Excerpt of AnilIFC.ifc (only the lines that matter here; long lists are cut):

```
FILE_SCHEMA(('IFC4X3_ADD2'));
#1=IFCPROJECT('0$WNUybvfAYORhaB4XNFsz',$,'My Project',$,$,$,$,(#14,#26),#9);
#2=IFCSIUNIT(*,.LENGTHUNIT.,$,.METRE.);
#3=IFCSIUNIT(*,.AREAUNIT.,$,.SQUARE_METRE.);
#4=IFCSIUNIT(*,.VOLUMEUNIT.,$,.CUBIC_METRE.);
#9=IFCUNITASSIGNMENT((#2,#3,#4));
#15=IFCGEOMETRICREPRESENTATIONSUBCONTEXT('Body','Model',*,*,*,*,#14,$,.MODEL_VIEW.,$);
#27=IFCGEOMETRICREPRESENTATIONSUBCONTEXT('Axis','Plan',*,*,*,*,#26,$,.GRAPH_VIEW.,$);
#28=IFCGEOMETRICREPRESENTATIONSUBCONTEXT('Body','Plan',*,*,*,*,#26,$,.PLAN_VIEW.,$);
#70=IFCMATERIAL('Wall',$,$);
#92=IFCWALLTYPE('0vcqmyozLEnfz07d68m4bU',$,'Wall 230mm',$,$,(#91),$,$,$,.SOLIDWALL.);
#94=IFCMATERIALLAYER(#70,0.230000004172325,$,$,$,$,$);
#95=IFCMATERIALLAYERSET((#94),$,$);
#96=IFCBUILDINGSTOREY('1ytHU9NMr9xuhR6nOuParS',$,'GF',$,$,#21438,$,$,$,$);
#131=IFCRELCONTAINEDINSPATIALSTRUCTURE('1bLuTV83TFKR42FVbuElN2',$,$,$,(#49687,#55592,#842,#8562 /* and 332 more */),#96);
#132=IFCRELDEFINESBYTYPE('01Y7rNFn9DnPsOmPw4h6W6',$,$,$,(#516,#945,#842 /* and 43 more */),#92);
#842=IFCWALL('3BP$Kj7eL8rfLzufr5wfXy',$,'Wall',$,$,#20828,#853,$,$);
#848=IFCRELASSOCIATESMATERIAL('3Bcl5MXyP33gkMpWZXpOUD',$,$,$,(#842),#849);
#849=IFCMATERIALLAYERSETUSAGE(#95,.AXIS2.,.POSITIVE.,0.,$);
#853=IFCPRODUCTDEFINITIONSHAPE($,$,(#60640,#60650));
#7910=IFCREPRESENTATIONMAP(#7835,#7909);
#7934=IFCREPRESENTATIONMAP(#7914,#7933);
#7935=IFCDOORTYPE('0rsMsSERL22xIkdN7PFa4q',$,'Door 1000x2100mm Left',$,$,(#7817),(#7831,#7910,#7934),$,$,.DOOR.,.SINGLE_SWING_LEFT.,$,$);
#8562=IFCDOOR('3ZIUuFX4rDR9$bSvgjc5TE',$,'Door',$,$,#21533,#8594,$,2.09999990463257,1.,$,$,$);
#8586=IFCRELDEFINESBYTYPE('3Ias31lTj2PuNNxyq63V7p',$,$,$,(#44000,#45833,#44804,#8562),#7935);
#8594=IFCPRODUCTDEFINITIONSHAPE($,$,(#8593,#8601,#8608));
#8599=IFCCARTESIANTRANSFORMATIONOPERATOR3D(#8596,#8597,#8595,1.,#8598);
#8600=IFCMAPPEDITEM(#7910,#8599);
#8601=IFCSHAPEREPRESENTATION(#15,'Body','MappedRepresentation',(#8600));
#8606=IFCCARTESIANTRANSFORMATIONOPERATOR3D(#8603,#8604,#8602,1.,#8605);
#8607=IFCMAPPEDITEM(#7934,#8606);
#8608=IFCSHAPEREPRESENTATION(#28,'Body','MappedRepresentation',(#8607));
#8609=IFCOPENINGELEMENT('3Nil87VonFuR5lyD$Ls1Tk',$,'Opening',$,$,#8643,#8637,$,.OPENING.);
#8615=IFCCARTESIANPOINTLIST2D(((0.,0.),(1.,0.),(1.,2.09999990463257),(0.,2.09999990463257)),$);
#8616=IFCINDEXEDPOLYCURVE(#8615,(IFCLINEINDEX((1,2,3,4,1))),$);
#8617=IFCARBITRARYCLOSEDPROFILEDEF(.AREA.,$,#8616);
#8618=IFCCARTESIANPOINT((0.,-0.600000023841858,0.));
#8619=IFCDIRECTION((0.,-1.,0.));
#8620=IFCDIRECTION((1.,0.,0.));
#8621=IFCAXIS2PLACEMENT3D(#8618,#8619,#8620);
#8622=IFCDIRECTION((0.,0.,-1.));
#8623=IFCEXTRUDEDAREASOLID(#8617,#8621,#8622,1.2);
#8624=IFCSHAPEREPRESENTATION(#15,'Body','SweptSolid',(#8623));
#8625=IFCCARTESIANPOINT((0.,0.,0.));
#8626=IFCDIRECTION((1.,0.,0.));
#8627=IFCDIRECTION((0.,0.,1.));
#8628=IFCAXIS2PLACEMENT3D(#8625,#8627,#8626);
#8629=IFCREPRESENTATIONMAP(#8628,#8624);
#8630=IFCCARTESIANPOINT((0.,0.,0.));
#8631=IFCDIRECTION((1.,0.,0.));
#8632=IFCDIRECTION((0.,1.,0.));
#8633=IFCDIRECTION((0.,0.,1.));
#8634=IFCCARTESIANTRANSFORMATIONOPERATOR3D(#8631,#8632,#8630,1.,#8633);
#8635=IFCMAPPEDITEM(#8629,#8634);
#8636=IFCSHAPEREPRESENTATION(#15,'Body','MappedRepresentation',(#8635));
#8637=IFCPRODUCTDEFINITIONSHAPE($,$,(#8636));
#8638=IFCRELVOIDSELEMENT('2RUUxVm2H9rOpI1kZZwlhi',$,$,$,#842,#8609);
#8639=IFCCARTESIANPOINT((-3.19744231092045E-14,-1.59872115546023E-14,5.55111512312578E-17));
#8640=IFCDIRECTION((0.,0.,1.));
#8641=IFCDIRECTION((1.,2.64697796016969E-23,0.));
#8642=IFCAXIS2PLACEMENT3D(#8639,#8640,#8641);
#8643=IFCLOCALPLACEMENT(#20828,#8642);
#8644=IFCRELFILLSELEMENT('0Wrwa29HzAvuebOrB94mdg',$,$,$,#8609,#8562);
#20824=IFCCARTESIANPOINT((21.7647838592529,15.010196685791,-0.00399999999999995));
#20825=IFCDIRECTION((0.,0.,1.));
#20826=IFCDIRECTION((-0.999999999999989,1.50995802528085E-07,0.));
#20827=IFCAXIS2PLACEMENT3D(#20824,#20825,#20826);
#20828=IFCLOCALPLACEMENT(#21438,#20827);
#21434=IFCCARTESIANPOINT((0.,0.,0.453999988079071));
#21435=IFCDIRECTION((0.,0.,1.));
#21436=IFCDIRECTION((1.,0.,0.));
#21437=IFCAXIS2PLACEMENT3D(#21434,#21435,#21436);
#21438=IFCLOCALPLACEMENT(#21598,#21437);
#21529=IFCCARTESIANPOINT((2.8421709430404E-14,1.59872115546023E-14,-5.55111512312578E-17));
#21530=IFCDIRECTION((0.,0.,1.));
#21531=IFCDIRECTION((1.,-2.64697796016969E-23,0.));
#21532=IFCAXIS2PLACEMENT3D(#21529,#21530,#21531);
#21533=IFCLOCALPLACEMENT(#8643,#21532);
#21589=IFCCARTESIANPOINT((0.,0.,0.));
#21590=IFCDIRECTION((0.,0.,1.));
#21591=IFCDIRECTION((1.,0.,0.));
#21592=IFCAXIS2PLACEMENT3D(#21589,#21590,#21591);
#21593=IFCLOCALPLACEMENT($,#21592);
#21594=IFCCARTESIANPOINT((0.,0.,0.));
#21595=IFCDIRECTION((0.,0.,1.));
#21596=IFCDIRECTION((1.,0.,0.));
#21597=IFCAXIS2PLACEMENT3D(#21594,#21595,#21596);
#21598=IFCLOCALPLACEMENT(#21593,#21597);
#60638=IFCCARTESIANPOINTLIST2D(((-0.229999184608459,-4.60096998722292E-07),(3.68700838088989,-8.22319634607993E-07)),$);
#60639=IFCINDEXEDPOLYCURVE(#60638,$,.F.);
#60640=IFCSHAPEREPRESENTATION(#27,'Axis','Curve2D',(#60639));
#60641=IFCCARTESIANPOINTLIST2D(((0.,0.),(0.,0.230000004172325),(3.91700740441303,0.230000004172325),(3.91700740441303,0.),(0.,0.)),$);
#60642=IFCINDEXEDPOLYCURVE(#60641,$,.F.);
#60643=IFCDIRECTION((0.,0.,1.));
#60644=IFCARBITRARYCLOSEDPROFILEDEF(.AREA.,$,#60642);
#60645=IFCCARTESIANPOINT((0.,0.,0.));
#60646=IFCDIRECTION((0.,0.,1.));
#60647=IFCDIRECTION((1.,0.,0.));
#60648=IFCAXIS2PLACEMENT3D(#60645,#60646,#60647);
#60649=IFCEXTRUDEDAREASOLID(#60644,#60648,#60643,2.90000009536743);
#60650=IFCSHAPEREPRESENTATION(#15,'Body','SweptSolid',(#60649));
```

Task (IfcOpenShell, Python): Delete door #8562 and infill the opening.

```python
import ifcopenshell
import ifcopenshell.api.feature
import ifcopenshell.api.root
import ifcopenshell.geom
import ifcopenshell.util.shape

model = ifcopenshell.open("AnilIFC.ifc")
settings = ifcopenshell.geom.settings()


def volume(element):
    """Net volume in cubic metres, openings subtracted."""
    shape = ifcopenshell.geom.create_shape(settings, element)
    return ifcopenshell.util.shape.get_volume(shape.geometry)


door = model.by_guid("3ZIUuFX4rDR9$bSvgjc5TE")
opening = door.FillsVoids[0].RelatingOpeningElement
wall = opening.VoidsElements[0].RelatingBuildingElement
before = volume(wall)

ifcopenshell.api.root.remove_product(model, product=door)
ifcopenshell.api.feature.remove_feature(model, feature=opening)

after = volume(wall)

print(f"wall volume {before:.3f} -> {after:.3f} m3")

model.write("AnilIFC_v2.ifc")
```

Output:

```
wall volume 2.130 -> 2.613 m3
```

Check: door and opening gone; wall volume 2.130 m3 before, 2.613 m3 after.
